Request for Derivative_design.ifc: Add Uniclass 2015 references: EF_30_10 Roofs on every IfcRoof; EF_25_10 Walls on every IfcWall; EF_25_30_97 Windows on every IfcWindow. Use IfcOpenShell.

First a look at what the model holds.

```python
import ifcopenshell

model = ifcopenshell.open("Derivative_design.ifc")
print(model.schema)
print("classifications:", [c.Name for c in model.by_type("IfcClassification")])
for ifc_class in ("IfcDoor", "IfcRoof", "IfcStair", "IfcWall", "IfcWindow"):
    print(ifc_class, len(model.by_type(ifc_class)))
```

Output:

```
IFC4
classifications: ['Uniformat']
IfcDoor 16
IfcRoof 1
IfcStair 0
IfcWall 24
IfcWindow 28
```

```python
import ifcopenshell
import ifcopenshell.api.classification

model = ifcopenshell.open("Derivative_design.ifc")

system = ifcopenshell.api.classification.add_classification(model, classification="Uniclass 2015")

codes = {
    "IfcRoof": ("EF_30_10", "Roofs"),
    "IfcWall": ("EF_25_10", "Walls"),
    "IfcWindow": ("EF_25_30_97", "Windows"),
}
for ifc_class, (code, name) in codes.items():
    products = model.by_type(ifc_class)
    ifcopenshell.api.classification.add_reference(
        model, products=products, classification=system, identification=code, name=name
    )
    print(code, len(products))

model.write("Derivative_design_updated.ifc")
```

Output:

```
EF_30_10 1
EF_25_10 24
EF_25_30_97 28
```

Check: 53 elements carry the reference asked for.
